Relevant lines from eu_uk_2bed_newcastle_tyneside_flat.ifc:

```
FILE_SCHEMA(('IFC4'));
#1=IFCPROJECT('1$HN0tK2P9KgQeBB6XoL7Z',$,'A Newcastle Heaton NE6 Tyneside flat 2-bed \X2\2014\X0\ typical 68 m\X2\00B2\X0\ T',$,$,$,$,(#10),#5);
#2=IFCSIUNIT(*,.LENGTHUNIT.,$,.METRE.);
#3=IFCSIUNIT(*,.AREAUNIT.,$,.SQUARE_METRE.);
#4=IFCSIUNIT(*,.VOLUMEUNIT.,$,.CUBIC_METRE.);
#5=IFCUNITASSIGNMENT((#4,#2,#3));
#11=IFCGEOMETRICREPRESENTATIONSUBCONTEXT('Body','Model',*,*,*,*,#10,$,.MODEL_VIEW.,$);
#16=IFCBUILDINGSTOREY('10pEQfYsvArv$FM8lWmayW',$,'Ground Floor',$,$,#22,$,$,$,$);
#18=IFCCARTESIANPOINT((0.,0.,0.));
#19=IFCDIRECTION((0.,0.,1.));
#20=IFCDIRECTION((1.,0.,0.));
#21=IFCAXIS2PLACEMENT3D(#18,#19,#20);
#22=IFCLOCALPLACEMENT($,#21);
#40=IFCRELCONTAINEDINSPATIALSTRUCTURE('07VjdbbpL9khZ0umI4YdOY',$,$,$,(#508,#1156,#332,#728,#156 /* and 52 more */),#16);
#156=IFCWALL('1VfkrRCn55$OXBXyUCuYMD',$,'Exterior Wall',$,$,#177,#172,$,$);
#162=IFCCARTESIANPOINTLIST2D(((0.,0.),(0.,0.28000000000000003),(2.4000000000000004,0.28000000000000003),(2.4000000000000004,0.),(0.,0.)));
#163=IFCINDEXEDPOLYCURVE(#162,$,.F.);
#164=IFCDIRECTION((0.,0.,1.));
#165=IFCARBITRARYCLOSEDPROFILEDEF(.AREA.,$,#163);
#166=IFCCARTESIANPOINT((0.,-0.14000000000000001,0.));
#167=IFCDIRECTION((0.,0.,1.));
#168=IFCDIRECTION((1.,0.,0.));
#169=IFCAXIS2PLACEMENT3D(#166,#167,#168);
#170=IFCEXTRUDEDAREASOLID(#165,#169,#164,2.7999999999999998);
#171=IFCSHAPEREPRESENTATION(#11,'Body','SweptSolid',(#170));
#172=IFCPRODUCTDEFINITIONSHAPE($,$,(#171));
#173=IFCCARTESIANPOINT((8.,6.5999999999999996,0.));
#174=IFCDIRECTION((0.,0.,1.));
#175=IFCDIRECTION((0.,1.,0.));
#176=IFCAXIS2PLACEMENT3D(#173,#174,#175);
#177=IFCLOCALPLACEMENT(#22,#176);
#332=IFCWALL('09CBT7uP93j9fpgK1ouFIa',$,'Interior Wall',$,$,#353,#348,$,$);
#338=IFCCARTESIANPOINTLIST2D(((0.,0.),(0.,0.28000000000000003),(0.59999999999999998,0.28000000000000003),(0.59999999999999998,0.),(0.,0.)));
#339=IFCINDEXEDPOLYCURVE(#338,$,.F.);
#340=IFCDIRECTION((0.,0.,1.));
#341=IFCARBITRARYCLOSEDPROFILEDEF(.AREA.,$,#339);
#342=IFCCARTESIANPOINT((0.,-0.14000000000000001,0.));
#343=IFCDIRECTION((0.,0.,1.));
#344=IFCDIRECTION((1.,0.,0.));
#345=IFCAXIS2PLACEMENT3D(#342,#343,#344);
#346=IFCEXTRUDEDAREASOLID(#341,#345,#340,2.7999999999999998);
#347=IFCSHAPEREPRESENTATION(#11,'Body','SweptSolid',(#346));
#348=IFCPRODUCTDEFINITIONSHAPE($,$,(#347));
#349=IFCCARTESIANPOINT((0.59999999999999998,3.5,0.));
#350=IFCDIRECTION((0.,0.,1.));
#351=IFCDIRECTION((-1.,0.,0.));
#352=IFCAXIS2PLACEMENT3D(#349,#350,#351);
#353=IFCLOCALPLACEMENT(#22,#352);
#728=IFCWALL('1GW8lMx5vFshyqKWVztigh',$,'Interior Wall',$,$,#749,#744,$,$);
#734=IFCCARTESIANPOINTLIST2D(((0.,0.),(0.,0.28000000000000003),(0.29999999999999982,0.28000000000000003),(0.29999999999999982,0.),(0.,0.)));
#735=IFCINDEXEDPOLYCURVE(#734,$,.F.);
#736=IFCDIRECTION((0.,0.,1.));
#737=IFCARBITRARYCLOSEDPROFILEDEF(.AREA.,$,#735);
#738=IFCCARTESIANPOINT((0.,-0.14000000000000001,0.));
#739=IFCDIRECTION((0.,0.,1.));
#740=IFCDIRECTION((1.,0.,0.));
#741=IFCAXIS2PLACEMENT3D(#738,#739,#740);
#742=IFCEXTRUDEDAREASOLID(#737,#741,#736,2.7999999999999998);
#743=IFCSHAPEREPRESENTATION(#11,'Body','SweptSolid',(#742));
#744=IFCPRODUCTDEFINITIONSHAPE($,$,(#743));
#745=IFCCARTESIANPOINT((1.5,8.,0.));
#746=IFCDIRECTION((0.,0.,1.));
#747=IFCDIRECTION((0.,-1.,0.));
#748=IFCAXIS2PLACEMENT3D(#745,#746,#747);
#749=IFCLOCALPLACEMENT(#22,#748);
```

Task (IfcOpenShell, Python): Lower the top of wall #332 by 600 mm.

```python
import ifcopenshell
import ifcopenshell.geom
import ifcopenshell.util.representation
import ifcopenshell.util.shape

model = ifcopenshell.open("eu_uk_2bed_newcastle_tyneside_flat.ifc")
settings = ifcopenshell.geom.settings()


def volume(element):
    """Net volume in cubic metres, openings subtracted."""
    shape = ifcopenshell.geom.create_shape(settings, element)
    return ifcopenshell.util.shape.get_volume(shape.geometry)


wall = model.by_guid("09CBT7uP93j9fpgK1ouFIa")
before = volume(wall)

body = ifcopenshell.util.representation.get_representation(wall, "Model", "Body")
solid = body.Items[0]
old_height = solid.Depth
solid.Depth -= 0.6
after = volume(wall)

print(f"height {old_height:g} -> {solid.Depth:g}, volume {before:.3f} -> {after:.3f} m3")

model.write("eu_uk_2bed_newcastle_tyneside_flat_rev.ifc")
```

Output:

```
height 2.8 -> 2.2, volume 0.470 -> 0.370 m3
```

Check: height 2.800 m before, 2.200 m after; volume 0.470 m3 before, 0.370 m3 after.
